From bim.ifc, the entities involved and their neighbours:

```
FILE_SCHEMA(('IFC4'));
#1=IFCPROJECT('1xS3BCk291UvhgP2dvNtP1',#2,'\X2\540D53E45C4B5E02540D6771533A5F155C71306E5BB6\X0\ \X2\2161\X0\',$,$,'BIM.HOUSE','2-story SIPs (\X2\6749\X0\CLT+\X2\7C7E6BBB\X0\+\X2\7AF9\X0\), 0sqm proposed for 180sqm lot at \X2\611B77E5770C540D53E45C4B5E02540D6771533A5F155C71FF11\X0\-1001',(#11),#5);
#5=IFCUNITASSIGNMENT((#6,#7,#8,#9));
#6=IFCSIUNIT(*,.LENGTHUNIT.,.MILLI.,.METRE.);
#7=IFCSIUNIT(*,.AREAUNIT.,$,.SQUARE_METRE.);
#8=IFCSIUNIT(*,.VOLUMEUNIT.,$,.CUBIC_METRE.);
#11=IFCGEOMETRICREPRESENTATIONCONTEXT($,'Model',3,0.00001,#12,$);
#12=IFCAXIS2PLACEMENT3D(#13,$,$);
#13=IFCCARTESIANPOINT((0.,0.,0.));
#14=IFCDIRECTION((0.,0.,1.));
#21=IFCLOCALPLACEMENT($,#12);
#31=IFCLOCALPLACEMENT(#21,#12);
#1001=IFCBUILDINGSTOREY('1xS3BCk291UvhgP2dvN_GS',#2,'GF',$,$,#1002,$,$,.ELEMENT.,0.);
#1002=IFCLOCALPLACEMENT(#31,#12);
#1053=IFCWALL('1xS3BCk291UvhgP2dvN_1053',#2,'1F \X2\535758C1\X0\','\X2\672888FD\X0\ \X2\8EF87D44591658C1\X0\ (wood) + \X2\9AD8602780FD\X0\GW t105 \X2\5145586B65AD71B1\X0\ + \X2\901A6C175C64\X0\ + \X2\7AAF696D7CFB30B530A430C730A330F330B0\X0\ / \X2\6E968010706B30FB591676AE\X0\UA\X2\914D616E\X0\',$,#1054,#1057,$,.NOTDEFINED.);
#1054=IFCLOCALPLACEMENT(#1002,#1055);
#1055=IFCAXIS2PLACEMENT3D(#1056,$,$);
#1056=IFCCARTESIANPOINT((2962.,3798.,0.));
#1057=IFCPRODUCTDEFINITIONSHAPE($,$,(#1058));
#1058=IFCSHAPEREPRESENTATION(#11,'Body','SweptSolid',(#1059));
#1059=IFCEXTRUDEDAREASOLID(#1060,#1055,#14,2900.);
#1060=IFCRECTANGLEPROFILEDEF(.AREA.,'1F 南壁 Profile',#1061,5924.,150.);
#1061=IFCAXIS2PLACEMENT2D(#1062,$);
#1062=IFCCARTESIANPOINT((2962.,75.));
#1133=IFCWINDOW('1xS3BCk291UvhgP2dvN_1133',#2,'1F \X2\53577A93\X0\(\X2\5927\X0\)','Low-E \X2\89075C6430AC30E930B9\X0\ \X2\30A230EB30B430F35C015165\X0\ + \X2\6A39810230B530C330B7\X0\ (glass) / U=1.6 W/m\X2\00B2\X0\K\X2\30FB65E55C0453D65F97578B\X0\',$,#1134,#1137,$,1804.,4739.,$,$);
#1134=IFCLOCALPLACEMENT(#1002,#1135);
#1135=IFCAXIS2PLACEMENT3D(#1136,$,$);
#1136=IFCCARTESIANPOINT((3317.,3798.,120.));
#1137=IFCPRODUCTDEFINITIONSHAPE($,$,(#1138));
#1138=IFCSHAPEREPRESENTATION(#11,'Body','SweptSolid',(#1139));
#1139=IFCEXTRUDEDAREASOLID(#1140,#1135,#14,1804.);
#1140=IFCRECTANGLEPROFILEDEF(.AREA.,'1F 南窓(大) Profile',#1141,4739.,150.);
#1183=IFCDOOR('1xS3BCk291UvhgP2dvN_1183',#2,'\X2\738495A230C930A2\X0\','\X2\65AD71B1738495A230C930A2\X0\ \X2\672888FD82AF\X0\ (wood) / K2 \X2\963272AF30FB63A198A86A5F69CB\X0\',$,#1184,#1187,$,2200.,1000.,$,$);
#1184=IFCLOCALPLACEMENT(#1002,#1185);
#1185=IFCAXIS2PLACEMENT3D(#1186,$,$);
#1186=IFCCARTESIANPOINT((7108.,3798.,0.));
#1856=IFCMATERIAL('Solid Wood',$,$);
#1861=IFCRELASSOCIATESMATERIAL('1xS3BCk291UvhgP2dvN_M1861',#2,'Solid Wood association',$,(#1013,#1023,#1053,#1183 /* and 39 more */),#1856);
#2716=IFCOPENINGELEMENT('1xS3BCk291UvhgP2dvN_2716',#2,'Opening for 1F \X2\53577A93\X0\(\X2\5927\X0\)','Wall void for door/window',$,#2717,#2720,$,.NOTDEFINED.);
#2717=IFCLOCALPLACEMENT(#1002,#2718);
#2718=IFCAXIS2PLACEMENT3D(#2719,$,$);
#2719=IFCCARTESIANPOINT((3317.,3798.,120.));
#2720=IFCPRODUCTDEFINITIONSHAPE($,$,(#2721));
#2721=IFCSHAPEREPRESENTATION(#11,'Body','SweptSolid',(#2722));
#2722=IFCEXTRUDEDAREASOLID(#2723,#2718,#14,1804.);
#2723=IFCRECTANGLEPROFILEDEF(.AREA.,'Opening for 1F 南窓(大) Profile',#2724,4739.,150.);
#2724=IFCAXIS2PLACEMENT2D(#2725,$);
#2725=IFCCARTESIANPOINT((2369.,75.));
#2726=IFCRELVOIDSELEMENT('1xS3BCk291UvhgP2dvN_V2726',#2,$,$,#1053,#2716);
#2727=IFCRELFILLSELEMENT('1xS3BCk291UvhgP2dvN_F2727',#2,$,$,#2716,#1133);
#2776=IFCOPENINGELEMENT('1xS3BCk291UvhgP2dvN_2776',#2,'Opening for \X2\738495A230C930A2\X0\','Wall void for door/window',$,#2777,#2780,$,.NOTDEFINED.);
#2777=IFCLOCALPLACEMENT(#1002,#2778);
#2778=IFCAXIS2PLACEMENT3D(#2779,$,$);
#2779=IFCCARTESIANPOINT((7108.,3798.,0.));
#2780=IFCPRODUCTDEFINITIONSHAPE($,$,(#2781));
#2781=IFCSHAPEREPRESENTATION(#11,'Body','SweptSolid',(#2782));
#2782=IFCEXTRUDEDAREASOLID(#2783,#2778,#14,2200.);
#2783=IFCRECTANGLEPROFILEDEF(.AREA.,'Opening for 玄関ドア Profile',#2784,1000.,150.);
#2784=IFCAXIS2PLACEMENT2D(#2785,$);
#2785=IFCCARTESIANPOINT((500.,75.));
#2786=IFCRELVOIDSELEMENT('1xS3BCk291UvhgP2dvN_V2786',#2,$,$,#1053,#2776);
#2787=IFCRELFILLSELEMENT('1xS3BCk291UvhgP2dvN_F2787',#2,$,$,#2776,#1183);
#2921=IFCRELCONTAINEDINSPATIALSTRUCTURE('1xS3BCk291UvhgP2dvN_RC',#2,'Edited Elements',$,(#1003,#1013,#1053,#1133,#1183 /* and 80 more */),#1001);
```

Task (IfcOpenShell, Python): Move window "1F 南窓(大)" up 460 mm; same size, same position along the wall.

```python
import numpy as np
import ifcopenshell
import ifcopenshell.api.geometry
import ifcopenshell.util.placement
import ifcopenshell.util.unit

model = ifcopenshell.open("bim.ifc")
unit_scale = ifcopenshell.util.unit.calculate_unit_scale(model)

window = model.by_guid("1xS3BCk291UvhgP2dvN_1133")
opening = window.FillsVoids[0].RelatingOpeningElement
dz = 460.0

shift = np.array([0.0, 0.0, dz])
# The window is not placed relative to its opening, so move both.
for product in (opening, window):
    matrix = ifcopenshell.util.placement.get_local_placement(product.ObjectPlacement)
    matrix[:3, 3] += shift
    ifcopenshell.api.geometry.edit_object_placement(model, product=product, matrix=matrix, is_si=False)

print(f"moved by {dz * unit_scale:+.3f} m")

model.write("bim_updated.ifc")
```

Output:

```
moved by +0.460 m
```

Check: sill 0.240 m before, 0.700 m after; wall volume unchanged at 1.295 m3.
